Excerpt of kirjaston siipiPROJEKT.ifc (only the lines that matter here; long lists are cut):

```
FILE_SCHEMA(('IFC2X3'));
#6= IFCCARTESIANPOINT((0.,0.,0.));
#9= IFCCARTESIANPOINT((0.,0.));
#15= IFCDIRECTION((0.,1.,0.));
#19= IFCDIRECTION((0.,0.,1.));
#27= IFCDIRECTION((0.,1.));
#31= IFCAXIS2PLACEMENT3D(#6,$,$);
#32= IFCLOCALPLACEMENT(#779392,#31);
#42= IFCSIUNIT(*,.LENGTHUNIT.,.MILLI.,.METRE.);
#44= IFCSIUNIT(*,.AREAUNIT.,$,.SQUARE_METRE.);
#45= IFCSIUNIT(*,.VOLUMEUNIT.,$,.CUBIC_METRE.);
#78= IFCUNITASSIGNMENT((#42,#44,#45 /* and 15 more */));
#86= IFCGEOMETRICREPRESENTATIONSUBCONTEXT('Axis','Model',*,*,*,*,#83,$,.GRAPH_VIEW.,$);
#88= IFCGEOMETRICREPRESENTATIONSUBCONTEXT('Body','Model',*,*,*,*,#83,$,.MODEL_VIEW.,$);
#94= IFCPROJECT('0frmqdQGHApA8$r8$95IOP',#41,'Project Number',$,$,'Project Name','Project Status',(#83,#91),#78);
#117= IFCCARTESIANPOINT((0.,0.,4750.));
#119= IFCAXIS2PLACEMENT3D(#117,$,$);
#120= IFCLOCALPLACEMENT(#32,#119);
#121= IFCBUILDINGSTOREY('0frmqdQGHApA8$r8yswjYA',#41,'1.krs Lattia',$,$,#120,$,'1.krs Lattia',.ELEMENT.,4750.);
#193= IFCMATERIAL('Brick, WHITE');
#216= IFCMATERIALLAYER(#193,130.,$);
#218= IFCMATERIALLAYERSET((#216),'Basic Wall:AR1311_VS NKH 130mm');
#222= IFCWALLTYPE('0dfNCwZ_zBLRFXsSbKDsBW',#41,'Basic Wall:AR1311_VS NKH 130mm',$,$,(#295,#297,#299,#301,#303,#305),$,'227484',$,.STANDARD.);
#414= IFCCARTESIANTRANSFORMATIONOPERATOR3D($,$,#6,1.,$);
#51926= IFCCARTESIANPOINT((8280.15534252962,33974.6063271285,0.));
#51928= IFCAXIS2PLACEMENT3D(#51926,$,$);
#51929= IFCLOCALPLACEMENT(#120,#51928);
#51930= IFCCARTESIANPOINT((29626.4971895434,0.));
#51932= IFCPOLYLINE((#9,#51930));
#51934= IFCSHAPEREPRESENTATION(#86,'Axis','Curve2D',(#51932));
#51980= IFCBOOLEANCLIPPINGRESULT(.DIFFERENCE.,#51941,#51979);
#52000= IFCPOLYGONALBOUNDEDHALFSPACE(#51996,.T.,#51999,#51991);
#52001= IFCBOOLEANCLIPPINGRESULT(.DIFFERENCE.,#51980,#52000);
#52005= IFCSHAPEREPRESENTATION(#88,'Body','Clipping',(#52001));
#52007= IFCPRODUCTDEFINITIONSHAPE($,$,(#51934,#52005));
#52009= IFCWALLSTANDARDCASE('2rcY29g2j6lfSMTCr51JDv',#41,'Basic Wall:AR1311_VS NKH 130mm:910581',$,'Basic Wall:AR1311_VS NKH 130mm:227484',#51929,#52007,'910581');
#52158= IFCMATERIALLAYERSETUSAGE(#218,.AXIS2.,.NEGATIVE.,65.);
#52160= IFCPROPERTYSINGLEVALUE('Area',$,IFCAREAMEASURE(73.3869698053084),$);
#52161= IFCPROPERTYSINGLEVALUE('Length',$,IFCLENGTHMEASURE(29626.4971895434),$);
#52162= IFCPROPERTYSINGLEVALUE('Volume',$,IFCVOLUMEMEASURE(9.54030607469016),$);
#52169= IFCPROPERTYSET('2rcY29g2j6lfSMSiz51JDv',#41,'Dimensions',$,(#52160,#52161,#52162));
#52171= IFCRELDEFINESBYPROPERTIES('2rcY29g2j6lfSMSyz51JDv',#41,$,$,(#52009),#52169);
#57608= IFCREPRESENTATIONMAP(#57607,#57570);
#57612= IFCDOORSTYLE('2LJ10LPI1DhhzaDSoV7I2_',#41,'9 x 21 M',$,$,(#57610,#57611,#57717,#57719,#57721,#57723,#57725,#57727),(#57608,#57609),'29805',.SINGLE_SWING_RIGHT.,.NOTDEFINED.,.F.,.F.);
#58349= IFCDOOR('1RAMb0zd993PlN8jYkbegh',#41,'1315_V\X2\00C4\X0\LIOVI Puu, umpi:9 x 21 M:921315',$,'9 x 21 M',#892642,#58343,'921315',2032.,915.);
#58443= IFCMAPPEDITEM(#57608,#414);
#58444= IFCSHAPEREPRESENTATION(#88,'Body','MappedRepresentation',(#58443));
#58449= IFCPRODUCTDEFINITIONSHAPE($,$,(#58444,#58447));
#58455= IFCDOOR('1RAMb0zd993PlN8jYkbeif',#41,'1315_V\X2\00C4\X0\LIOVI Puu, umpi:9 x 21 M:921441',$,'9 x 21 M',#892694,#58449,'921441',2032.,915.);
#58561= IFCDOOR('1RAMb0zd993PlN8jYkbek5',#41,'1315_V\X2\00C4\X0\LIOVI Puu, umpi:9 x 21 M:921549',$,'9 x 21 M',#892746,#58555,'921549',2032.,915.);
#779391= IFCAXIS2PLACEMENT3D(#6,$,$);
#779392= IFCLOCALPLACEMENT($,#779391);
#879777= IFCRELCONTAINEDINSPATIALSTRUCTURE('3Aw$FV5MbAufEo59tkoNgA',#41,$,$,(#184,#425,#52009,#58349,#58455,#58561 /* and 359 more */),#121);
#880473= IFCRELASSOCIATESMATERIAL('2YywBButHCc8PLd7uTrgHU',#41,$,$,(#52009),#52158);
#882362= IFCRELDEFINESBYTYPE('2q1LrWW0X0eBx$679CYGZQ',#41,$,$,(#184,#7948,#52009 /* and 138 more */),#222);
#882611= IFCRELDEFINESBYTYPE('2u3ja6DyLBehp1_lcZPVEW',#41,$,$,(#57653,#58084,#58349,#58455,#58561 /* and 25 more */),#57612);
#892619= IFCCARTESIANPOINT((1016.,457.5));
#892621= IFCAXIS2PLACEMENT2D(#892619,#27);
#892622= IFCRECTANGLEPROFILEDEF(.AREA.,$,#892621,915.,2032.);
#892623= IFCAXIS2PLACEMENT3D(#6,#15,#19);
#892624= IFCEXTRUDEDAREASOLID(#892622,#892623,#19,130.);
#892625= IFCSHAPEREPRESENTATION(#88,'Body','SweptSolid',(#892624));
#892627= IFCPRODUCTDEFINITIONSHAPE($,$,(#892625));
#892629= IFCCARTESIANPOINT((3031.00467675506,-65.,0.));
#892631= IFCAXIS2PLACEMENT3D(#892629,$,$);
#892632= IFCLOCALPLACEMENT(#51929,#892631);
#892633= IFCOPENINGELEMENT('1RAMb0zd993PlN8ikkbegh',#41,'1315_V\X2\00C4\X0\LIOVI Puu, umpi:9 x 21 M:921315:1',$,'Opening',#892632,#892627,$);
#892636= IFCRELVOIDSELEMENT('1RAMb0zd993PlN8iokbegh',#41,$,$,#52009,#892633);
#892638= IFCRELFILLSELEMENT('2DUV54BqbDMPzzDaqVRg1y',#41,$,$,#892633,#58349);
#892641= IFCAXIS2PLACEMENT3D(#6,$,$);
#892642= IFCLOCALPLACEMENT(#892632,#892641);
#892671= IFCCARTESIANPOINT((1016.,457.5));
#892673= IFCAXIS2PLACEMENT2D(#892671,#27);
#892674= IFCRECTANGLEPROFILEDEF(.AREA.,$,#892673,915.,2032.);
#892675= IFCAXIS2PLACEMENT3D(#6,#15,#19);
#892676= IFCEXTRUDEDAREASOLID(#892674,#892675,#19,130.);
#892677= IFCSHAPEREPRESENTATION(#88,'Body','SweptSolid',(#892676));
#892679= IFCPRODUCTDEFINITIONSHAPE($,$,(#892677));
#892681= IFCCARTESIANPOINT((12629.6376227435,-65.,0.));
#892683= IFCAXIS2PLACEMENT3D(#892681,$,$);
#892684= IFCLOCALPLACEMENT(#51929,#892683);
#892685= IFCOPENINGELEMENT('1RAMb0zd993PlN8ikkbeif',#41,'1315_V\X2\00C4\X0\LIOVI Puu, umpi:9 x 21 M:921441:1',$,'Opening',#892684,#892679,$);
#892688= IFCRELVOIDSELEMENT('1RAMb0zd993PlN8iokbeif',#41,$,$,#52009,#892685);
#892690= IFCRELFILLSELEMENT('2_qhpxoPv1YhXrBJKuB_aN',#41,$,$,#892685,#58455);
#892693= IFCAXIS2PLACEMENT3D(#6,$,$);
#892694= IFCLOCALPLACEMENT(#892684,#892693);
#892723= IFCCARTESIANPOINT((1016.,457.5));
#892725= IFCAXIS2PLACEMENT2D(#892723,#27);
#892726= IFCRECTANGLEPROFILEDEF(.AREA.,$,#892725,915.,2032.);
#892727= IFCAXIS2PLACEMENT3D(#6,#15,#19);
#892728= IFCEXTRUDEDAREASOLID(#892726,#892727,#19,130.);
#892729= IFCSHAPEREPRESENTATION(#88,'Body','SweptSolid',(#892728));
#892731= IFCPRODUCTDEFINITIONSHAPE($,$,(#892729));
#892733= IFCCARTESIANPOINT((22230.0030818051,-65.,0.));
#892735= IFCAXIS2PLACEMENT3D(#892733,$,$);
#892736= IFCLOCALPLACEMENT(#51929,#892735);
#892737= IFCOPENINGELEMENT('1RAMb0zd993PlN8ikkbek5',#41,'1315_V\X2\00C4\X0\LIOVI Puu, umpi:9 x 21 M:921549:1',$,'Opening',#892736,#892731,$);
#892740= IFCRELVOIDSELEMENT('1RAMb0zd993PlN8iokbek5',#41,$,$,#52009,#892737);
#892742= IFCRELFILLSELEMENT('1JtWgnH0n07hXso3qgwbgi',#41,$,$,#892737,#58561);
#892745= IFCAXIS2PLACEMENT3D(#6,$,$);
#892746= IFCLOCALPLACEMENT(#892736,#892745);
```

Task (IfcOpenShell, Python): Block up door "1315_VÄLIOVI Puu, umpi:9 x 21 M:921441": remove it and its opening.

```python
import ifcopenshell
import ifcopenshell.api.feature
import ifcopenshell.api.pset
import ifcopenshell.api.root
import ifcopenshell.geom
import ifcopenshell.util.element
import ifcopenshell.util.shape
import ifcopenshell.util.unit

model = ifcopenshell.open("kirjaston siipiPROJEKT.ifc")
area_scale = ifcopenshell.util.unit.calculate_unit_scale(model, "AREAUNIT")
volume_scale = ifcopenshell.util.unit.calculate_unit_scale(model, "VOLUMEUNIT")
settings = ifcopenshell.geom.settings()


def volume(element):
    """Net volume in cubic metres, openings subtracted."""
    shape = ifcopenshell.geom.create_shape(settings, element)
    return ifcopenshell.util.shape.get_volume(shape.geometry)


door = model.by_guid("1RAMb0zd993PlN8jYkbeif")
opening = door.FillsVoids[0].RelatingOpeningElement
wall = opening.VoidsElements[0].RelatingBuildingElement
before = volume(wall)

ifcopenshell.api.root.remove_product(model, product=door)
ifcopenshell.api.feature.remove_feature(model, feature=opening)

after = volume(wall)
thickness = 0.13  # wall thickness in metres

# Update the wall's stored quantities.
pset = model.by_id(ifcopenshell.util.element.get_pset(wall, "Dimensions", should_inherit=False)["id"])
ifcopenshell.api.pset.edit_pset(model, pset=pset, properties={
    "Area": model.create_entity("IfcAreaMeasure", after / thickness / area_scale),
    "Volume": model.create_entity("IfcVolumeMeasure", after / volume_scale),
})

print(f"wall volume {before:.3f} -> {after:.3f} m3")

model.write("kirjaston siipiPROJEKT_v2.ifc")
```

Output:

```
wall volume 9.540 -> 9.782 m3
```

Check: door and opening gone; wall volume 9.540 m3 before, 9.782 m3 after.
